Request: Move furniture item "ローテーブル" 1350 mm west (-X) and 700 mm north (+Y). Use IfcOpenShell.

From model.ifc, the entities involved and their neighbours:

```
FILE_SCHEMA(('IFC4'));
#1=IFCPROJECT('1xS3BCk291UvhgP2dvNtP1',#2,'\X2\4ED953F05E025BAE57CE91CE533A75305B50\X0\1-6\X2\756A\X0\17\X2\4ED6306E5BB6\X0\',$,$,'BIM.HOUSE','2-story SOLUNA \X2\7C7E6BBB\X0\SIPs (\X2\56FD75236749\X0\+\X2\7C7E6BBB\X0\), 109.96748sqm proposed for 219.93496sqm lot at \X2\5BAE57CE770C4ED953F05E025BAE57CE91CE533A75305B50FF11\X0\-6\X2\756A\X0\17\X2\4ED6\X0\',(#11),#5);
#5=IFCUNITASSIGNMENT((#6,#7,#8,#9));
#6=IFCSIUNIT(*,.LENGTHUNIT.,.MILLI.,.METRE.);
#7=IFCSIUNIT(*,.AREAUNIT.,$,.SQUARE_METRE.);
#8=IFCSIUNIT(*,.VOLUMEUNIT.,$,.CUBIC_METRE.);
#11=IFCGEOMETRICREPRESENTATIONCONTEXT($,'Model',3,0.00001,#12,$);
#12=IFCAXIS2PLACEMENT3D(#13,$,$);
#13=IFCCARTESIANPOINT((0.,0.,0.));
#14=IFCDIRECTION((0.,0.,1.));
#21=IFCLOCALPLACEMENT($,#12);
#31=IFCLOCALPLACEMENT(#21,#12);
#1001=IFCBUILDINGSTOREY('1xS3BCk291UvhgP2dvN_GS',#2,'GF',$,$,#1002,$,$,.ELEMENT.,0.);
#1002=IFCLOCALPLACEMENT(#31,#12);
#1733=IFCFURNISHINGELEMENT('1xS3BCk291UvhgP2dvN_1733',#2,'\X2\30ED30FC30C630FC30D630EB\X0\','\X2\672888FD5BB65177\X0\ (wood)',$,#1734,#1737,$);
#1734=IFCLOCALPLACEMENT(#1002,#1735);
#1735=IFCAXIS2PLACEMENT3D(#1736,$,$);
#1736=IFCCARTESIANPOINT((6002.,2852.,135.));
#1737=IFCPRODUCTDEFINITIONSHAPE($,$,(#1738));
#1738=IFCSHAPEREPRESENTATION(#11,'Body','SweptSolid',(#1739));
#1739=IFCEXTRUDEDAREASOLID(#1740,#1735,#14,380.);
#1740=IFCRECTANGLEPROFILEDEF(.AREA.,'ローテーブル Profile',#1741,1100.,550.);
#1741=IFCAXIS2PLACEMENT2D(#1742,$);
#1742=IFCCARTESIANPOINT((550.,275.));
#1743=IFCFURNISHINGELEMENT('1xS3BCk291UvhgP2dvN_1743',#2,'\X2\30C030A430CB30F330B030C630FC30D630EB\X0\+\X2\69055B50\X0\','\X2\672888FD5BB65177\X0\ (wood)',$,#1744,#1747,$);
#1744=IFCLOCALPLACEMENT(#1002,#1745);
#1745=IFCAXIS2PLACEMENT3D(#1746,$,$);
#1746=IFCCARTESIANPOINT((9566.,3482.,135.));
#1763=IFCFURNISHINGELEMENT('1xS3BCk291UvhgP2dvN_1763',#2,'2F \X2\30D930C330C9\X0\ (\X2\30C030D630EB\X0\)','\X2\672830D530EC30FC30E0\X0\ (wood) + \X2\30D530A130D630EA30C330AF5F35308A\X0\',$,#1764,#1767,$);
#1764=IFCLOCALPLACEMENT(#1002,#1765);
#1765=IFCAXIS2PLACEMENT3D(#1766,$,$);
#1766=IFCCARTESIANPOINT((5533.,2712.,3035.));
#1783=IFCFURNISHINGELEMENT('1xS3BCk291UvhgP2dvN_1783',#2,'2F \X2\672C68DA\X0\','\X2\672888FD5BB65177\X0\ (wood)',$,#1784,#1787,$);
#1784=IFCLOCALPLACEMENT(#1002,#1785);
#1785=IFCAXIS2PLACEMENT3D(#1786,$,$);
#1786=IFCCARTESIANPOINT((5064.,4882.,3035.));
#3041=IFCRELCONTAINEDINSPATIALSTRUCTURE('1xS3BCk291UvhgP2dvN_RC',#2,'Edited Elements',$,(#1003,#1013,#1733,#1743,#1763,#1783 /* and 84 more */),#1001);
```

```python
import ifcopenshell
import ifcopenshell.api.geometry
import ifcopenshell.util.placement
import ifcopenshell.util.unit

model = ifcopenshell.open("model.ifc")
unit_scale = ifcopenshell.util.unit.calculate_unit_scale(model)

item = model.by_guid("1xS3BCk291UvhgP2dvN_1733")
matrix = ifcopenshell.util.placement.get_local_placement(item.ObjectPlacement)
matrix[0, 3] -= 1.35 / unit_scale
matrix[1, 3] += 0.7 / unit_scale
ifcopenshell.api.geometry.edit_object_placement(model, product=item, matrix=matrix, is_si=False)

print(ifcopenshell.util.placement.get_local_placement(item.ObjectPlacement).round(3) + 0.0)

model.write("model_edited.ifc")
```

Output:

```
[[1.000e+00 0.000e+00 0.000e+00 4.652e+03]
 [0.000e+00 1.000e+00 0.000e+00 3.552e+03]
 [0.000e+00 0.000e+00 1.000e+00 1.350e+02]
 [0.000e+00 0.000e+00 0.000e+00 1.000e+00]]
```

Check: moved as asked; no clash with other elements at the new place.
